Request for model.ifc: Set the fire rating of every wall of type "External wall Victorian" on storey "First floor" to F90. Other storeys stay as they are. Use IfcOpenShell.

First a look at what the model holds.

```python
import ifcopenshell
import ifcopenshell.util.element

model = ifcopenshell.open("model.ifc")
print(model.schema)
storey = next(s for s in model.by_type("IfcBuildingStorey") if s.Name == "First floor")
walls = [e for e in ifcopenshell.util.element.get_decomposition(storey) if e.is_a("IfcWall")]
seen = {}
for e in walls:
    element_type = ifcopenshell.util.element.get_type(e)
    key = (element_type.Name if element_type != e and element_type else None, ifcopenshell.util.element.get_pset(e, "Pset_WallCommon", "FireRating"))
    seen[key] = seen.get(key, 0) + 1
for (name, value), count in sorted(seen.items(), key=str):
    print(count, "x", name, "|", value)
```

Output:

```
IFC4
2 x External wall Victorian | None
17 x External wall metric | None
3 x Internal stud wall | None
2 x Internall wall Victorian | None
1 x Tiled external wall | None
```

```python
import ifcopenshell
import ifcopenshell.api.pset
import ifcopenshell.util.element

model = ifcopenshell.open("model.ifc")

storey = next(s for s in model.by_type("IfcBuildingStorey") if s.Name == "First floor")
walls = [e for e in ifcopenshell.util.element.get_decomposition(storey) if e.is_a("IfcWall")]

count = 0
for e in walls:
    element_type = ifcopenshell.util.element.get_type(e)
    if element_type in (None, e) or element_type.Name != "External wall Victorian":
        continue
    # add_pset returns the element's existing set when there is one.
    pset = ifcopenshell.api.pset.add_pset(model, product=e, name="Pset_WallCommon")
    ifcopenshell.api.pset.edit_pset(model, pset=pset, properties={"FireRating": "F90"})
    count += 1

print(count, "walls updated")

model.write("model_v2.ifc")
```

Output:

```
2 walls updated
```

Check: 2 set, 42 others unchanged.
